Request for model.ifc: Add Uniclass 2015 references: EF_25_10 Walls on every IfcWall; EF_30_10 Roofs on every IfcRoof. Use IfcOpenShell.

First a look at what the model holds.

```python
import ifcopenshell

model = ifcopenshell.open("model.ifc")
print(model.schema)
print("classifications:", [c.Name for c in model.by_type("IfcClassification")])
for ifc_class in ("IfcDoor", "IfcRoof", "IfcStair", "IfcWall", "IfcWindow"):
    print(ifc_class, len(model.by_type(ifc_class)))
```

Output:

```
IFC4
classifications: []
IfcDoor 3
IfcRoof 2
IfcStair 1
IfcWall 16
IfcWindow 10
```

```python
import ifcopenshell
import ifcopenshell.api.classification

model = ifcopenshell.open("model.ifc")

system = ifcopenshell.api.classification.add_classification(model, classification="Uniclass 2015")

codes = {
    "IfcWall": ("EF_25_10", "Walls"),
    "IfcRoof": ("EF_30_10", "Roofs"),
}
for ifc_class, (code, name) in codes.items():
    products = model.by_type(ifc_class)
    ifcopenshell.api.classification.add_reference(
        model, products=products, classification=system, identification=code, name=name
    )
    print(code, len(products))

model.write("model_v2.ifc")
```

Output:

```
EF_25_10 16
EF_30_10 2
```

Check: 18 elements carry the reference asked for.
